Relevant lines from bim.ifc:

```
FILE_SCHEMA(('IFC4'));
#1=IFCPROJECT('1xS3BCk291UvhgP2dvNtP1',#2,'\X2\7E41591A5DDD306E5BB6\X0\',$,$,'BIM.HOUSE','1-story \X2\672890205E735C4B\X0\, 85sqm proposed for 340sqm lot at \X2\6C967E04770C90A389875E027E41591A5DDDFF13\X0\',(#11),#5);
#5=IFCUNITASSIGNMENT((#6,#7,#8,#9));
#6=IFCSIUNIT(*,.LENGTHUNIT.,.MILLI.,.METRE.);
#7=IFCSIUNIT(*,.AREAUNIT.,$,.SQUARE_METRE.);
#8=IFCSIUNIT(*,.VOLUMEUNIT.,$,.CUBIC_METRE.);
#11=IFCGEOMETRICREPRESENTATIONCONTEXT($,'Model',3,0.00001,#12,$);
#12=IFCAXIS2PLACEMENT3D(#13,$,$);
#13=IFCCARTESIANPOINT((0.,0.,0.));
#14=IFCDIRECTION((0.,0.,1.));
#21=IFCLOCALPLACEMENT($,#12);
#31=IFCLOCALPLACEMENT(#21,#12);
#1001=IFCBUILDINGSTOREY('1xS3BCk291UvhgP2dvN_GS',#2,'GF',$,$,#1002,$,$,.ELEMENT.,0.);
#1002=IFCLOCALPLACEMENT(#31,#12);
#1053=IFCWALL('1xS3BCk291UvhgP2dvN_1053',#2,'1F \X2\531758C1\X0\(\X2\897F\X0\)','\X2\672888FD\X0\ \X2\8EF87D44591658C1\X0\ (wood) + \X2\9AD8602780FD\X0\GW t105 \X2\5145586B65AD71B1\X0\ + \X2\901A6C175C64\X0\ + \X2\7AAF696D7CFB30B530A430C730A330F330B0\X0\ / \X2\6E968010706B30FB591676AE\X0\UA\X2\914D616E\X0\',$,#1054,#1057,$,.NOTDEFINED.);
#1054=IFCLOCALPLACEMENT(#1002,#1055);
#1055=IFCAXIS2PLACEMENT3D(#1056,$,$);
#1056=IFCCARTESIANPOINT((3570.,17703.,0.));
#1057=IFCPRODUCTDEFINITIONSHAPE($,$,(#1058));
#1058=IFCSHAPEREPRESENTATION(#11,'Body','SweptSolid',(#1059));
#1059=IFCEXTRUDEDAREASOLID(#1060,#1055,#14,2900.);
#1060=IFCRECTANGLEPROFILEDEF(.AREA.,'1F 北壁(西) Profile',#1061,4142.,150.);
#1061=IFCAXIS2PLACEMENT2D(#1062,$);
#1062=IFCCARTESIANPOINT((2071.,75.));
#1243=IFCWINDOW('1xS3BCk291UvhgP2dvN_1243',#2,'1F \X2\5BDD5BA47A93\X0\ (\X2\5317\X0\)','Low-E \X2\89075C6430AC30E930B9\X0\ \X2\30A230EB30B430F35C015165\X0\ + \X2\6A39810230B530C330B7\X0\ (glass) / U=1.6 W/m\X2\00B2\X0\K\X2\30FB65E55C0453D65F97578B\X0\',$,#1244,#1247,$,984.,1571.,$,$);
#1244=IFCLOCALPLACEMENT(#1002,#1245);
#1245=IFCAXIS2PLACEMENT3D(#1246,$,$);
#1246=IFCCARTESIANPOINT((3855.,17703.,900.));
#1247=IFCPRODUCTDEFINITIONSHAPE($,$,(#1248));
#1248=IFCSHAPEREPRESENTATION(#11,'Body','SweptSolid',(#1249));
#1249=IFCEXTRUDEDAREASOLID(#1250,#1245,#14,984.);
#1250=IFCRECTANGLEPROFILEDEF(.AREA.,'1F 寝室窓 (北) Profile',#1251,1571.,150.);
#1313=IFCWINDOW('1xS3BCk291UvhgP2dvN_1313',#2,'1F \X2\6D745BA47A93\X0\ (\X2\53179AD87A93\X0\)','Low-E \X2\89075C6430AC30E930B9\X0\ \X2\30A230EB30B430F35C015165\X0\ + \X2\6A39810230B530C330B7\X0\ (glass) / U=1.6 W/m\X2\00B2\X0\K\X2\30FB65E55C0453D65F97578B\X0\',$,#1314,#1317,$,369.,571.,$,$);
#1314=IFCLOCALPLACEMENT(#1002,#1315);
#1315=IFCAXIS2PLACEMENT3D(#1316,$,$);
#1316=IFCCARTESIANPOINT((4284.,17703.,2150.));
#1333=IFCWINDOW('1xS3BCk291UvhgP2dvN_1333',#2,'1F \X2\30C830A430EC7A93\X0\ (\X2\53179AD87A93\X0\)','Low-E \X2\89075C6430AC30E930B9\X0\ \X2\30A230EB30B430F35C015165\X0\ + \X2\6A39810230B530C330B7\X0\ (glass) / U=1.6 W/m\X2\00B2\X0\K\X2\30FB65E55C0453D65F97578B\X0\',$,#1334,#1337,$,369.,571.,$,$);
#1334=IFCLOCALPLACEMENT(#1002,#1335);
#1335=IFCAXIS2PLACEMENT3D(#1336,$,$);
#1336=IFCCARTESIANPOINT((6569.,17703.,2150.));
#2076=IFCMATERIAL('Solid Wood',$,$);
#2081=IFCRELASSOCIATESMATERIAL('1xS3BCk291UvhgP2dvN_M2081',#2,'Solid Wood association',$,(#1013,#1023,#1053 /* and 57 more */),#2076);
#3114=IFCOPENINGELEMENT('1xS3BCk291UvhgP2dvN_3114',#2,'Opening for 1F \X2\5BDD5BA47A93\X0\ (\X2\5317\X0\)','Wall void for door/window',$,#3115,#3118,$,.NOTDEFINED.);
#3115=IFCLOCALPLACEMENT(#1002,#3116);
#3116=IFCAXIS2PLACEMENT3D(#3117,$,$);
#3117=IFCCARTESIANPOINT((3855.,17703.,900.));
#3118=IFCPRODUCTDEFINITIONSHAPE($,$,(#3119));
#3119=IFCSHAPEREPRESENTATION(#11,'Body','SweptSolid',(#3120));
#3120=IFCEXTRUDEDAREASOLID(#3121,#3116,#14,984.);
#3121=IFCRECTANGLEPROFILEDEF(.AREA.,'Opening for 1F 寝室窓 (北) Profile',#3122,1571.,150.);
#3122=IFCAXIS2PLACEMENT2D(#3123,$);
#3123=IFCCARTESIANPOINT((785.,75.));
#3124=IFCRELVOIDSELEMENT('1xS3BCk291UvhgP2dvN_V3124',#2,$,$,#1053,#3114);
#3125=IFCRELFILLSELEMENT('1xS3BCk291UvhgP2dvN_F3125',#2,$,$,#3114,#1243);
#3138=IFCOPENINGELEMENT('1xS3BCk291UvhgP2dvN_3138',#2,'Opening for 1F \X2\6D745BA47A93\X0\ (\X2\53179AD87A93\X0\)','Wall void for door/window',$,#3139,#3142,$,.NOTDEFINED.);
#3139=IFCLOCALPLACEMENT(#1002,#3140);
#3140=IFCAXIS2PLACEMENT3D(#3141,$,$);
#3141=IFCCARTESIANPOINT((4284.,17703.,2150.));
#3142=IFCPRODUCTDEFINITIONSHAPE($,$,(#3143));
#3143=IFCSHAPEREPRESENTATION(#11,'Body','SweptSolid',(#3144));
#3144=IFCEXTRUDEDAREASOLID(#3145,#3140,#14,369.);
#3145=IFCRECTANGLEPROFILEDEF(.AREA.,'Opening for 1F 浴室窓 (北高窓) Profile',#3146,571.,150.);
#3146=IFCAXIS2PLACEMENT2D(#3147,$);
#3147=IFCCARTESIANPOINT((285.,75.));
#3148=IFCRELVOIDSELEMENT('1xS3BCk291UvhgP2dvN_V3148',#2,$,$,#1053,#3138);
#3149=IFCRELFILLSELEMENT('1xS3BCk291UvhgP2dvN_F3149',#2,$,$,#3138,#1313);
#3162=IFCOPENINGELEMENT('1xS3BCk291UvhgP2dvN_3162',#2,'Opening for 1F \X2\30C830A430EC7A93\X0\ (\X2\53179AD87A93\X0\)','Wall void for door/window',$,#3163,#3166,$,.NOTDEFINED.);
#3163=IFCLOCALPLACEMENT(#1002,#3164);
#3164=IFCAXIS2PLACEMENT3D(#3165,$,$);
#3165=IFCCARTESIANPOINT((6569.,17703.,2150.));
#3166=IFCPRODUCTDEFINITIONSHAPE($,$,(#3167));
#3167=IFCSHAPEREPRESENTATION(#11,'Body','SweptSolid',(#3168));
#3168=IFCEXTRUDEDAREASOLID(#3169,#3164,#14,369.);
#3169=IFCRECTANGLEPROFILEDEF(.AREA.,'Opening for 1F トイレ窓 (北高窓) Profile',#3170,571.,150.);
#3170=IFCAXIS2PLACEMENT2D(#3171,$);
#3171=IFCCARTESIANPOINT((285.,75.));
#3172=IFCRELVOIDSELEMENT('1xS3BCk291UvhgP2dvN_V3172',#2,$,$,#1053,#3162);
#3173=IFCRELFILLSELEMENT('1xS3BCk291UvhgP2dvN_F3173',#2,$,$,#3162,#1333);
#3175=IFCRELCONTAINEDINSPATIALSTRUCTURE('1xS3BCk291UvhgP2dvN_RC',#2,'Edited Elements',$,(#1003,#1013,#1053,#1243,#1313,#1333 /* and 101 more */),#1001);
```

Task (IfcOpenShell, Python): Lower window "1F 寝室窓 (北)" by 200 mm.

```python
import numpy as np
import ifcopenshell
import ifcopenshell.api.geometry
import ifcopenshell.util.placement
import ifcopenshell.util.unit

model = ifcopenshell.open("bim.ifc")
unit_scale = ifcopenshell.util.unit.calculate_unit_scale(model)

window = model.by_guid("1xS3BCk291UvhgP2dvN_1243")
opening = window.FillsVoids[0].RelatingOpeningElement
dz = -0.2 / unit_scale

shift = np.array([0.0, 0.0, dz])
# The window is not placed relative to its opening, so move both.
for product in (opening, window):
    matrix = ifcopenshell.util.placement.get_local_placement(product.ObjectPlacement)
    matrix[:3, 3] += shift
    ifcopenshell.api.geometry.edit_object_placement(model, product=product, matrix=matrix, is_si=False)

print(f"moved by {dz * unit_scale:+.3f} m")

model.write("bim_v2.ifc")
```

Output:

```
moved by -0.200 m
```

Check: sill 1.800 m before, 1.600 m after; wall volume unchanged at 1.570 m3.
